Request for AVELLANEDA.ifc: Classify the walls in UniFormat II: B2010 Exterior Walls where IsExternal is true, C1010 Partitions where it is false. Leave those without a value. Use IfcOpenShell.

First a look at what the model holds.

```python
import ifcopenshell
import ifcopenshell.util.element

model = ifcopenshell.open("AVELLANEDA.ifc")
print(model.schema)
print("classifications:", [c.Name for c in model.by_type("IfcClassification")])
values = [ifcopenshell.util.element.get_pset(e, "Pset_WallCommon", "IsExternal") for e in model.by_type("IfcWall")]
for value in (True, False, None):
    print("IsExternal", value, values.count(value))
```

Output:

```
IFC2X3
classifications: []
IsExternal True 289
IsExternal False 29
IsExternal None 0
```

```python
import ifcopenshell
import ifcopenshell.api.classification
import ifcopenshell.util.element

model = ifcopenshell.open("AVELLANEDA.ifc")

# IFC2X3 requires Source and Edition and has no link from the project to the system.
system = model.create_entity("IfcClassification", Source="ASTM", Edition="E1557", Name="UniFormat II")

walls = model.by_type("IfcWall")
external = {e: ifcopenshell.util.element.get_pset(e, "Pset_WallCommon", "IsExternal") for e in walls}
for flag, code, name in ((True, "B2010", "Exterior Walls"), (False, "C1010", "Partitions")):
    products = [e for e in walls if external[e] is flag]
    ifcopenshell.api.classification.add_reference(
        model, products=products, classification=system, identification=code, name=name
    )
    print(code, len(products))

model.write("AVELLANEDA-out.ifc")
```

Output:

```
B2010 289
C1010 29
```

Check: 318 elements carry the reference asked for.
